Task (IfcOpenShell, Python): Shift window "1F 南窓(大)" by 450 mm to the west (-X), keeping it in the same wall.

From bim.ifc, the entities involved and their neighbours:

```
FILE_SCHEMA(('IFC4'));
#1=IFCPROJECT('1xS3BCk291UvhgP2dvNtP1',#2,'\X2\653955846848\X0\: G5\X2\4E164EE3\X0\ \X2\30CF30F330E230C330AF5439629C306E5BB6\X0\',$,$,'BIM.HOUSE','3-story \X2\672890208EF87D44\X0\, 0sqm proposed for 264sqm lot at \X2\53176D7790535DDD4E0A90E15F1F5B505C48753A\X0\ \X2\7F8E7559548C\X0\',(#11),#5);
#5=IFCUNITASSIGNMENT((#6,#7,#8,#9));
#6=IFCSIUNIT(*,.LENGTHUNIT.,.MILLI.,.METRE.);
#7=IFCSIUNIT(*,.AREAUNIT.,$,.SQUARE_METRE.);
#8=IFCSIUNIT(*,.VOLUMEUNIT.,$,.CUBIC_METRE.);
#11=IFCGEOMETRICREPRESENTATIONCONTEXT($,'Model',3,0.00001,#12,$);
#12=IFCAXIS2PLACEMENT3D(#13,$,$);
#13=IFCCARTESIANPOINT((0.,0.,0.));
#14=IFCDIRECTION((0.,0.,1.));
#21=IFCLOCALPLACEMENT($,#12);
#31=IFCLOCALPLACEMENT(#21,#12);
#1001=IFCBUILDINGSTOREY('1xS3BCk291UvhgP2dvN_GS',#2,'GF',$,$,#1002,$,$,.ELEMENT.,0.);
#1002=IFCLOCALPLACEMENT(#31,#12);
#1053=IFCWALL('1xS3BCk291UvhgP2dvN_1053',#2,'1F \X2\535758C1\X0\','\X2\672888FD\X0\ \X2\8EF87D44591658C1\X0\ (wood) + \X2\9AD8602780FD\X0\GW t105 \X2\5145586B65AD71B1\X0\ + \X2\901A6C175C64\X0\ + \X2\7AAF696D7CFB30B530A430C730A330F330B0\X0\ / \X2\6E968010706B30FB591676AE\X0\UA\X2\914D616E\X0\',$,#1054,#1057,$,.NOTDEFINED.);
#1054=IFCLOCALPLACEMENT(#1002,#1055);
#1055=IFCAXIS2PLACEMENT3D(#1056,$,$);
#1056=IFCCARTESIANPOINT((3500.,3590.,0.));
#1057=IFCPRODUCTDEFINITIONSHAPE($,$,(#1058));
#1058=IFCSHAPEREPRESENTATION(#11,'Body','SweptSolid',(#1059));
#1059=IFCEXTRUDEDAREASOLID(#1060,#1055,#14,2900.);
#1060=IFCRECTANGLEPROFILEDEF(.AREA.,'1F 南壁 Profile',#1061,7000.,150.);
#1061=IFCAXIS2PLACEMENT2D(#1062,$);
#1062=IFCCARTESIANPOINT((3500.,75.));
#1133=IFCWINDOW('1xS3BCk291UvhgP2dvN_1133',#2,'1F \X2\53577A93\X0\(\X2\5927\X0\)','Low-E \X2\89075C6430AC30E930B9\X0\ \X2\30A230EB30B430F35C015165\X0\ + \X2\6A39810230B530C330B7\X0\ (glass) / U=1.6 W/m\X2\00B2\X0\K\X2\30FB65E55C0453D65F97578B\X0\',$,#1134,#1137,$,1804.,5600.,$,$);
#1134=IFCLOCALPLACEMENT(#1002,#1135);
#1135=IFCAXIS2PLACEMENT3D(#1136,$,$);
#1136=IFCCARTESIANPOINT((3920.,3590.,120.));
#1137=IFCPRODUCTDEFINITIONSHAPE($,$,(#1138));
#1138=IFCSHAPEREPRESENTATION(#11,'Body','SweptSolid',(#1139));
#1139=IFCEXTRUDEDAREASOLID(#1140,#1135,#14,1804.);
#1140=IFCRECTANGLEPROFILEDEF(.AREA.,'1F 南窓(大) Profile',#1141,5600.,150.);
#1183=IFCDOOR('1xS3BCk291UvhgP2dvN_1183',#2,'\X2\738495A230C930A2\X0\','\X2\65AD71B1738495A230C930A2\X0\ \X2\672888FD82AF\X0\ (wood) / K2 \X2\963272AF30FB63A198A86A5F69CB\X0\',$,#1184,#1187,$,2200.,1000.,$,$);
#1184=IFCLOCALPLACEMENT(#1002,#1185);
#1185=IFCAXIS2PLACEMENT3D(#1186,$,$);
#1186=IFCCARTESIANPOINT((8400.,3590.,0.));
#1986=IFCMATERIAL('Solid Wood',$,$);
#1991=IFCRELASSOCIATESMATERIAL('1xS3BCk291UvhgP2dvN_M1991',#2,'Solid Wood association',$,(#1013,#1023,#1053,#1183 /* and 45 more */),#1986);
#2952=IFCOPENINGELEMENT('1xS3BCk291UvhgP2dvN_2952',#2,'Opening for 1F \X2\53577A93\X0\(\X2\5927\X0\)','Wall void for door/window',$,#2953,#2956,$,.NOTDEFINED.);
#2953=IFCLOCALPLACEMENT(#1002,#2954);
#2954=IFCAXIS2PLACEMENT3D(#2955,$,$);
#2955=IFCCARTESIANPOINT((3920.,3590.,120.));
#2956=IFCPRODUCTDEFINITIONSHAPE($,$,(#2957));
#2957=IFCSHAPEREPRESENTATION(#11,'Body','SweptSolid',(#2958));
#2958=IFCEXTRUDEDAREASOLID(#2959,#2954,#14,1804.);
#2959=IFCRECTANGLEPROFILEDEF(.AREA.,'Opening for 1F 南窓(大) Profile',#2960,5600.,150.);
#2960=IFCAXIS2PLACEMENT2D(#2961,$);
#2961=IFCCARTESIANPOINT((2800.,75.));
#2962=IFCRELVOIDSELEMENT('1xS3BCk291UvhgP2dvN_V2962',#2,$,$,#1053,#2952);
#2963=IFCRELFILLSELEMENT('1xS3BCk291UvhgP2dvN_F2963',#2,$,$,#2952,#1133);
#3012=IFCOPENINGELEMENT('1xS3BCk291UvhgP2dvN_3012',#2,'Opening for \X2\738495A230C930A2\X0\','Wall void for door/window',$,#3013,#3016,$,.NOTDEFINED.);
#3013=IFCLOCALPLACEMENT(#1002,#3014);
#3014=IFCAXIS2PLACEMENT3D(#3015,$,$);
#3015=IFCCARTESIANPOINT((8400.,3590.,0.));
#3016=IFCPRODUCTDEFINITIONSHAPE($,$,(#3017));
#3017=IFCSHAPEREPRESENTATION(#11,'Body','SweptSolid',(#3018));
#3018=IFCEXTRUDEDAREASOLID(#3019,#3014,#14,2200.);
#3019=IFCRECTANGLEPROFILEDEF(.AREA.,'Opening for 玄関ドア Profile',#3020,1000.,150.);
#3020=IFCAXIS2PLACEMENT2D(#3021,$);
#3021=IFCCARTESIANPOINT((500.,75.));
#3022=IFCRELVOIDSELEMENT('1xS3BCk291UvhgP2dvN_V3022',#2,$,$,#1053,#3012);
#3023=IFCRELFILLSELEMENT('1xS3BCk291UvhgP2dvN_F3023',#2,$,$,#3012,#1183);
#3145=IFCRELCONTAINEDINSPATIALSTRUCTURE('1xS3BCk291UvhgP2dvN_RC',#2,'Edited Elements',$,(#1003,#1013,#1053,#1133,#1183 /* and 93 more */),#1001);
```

```python
import ifcopenshell
import ifcopenshell.api.geometry
import ifcopenshell.util.placement

model = ifcopenshell.open("bim.ifc")

window = model.by_guid("1xS3BCk291UvhgP2dvN_1133")
opening = window.FillsVoids[0].RelatingOpeningElement
wall = opening.VoidsElements[0].RelatingBuildingElement

wall_matrix = ifcopenshell.util.placement.get_local_placement(wall.ObjectPlacement)
shift = wall_matrix[:3, 0] * -450.0
before = ifcopenshell.util.placement.get_local_placement(window.ObjectPlacement)[:3, 3].copy()

# The window is not placed relative to its opening, so move both.
for product in (opening, window):
    matrix = ifcopenshell.util.placement.get_local_placement(product.ObjectPlacement)
    matrix[:3, 3] += shift
    ifcopenshell.api.geometry.edit_object_placement(model, product=product, matrix=matrix, is_si=False)

after = ifcopenshell.util.placement.get_local_placement(window.ObjectPlacement)[:3, 3]
print("window moved by", (after - before).round(3) + 0.0)

model.write("bim_v2.ifc")
```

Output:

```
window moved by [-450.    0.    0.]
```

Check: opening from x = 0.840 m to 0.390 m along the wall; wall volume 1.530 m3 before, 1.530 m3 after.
